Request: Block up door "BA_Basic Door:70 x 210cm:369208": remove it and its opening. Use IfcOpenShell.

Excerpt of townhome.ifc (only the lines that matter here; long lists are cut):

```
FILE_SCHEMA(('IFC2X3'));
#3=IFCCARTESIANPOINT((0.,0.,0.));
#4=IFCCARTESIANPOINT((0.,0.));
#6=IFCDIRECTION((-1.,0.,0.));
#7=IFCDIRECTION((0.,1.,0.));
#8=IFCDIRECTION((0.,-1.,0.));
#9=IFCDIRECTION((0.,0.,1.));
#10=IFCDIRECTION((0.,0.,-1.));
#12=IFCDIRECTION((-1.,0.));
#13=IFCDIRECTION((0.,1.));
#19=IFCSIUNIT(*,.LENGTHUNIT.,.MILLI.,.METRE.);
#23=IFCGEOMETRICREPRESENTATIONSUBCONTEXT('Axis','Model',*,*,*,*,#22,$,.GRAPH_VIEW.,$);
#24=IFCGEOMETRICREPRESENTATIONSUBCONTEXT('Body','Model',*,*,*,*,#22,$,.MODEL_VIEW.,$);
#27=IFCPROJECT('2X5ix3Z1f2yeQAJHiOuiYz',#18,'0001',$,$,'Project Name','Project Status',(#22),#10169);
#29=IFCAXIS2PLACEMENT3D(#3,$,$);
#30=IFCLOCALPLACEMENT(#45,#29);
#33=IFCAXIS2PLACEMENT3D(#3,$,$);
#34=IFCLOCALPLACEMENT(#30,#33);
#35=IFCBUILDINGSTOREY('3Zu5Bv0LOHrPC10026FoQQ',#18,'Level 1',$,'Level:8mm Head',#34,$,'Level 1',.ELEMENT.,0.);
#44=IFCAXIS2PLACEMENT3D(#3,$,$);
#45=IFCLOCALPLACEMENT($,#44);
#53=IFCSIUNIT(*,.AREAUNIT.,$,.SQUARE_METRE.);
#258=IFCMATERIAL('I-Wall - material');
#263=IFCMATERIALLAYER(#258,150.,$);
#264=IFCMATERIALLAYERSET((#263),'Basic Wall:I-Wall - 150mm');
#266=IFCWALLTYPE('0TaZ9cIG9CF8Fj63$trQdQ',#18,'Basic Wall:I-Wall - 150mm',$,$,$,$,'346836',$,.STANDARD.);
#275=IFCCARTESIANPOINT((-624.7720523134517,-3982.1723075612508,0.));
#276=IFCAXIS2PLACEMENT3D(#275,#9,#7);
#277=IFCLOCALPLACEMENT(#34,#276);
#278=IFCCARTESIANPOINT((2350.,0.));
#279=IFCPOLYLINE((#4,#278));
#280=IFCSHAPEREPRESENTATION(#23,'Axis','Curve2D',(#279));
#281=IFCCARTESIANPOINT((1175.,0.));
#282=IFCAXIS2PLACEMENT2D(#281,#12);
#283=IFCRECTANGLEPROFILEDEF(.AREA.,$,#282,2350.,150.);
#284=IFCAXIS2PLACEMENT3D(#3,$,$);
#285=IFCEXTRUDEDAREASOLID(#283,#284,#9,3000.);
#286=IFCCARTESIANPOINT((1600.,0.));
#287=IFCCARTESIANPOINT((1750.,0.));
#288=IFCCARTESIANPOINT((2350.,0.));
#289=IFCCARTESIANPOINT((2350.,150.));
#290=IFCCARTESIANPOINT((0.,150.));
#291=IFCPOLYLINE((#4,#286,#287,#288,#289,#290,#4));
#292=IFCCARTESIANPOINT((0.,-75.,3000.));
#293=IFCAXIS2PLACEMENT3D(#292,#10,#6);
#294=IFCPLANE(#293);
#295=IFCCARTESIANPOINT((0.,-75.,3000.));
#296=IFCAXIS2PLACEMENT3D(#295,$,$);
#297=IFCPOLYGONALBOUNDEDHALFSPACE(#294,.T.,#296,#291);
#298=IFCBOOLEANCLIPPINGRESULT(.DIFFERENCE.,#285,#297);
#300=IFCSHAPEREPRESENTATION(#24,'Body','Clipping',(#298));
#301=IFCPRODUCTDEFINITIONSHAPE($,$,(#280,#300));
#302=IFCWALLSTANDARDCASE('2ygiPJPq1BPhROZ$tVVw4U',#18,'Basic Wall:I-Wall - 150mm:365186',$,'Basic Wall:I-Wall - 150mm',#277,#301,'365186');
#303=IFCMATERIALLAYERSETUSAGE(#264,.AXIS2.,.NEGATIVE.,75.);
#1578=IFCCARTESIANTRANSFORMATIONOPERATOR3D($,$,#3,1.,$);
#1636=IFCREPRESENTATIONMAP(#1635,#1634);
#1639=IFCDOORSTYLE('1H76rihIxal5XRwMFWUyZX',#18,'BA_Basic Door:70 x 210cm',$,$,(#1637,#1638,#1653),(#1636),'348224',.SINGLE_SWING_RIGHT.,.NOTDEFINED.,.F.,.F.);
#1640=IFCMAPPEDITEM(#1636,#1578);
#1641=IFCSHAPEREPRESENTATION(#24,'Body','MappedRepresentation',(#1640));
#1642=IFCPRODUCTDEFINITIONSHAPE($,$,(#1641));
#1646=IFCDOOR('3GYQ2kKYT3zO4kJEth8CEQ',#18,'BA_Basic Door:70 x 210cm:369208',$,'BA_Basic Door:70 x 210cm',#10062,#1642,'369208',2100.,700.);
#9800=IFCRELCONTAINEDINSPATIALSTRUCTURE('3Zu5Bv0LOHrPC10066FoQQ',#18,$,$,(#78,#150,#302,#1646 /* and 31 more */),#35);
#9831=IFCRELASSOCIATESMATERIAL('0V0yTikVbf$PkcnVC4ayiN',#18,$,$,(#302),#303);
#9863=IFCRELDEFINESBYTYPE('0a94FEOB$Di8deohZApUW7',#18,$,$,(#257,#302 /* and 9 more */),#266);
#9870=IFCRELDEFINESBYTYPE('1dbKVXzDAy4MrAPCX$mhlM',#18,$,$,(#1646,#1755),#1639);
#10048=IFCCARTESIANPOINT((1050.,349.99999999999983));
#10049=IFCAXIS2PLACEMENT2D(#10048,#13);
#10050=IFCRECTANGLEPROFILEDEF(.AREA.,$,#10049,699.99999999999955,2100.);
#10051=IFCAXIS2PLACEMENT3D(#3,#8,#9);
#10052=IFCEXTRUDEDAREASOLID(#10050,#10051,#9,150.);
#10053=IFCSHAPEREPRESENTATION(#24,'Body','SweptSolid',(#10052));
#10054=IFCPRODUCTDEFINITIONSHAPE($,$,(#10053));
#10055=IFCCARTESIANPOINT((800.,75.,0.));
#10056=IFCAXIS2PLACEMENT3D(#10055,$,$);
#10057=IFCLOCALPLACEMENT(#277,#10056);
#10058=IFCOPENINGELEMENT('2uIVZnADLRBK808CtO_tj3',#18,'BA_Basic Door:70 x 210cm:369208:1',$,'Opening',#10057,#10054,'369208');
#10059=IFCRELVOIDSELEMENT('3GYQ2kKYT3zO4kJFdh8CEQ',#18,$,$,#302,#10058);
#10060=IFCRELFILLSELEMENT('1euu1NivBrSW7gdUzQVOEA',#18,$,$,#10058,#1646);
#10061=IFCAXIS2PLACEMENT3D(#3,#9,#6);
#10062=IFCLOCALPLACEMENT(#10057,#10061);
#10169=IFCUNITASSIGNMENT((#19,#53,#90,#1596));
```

```python
import ifcopenshell
import ifcopenshell.api.feature
import ifcopenshell.api.root
import ifcopenshell.geom
import ifcopenshell.util.shape

model = ifcopenshell.open("townhome.ifc")
settings = ifcopenshell.geom.settings()


def volume(element):
    """Net volume in cubic metres, openings subtracted."""
    shape = ifcopenshell.geom.create_shape(settings, element)
    return ifcopenshell.util.shape.get_volume(shape.geometry)


door = model.by_guid("3GYQ2kKYT3zO4kJEth8CEQ")
opening = door.FillsVoids[0].RelatingOpeningElement
wall = opening.VoidsElements[0].RelatingBuildingElement
before = volume(wall)

ifcopenshell.api.root.remove_product(model, product=door)
ifcopenshell.api.feature.remove_feature(model, feature=opening)

after = volume(wall)

print(f"wall volume {before:.3f} -> {after:.3f} m3")

model.write("townhome_rev.ifc")
```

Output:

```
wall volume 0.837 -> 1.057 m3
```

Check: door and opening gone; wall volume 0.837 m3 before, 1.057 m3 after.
